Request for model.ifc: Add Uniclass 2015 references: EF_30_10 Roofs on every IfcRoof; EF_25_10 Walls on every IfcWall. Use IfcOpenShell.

First a look at what the model holds.

```python
import ifcopenshell

model = ifcopenshell.open("model.ifc")
print(model.schema)
print("classifications:", [c.Name for c in model.by_type("IfcClassification")])
for ifc_class in ("IfcDoor", "IfcRoof", "IfcStair", "IfcWall", "IfcWindow"):
    print(ifc_class, len(model.by_type(ifc_class)))
```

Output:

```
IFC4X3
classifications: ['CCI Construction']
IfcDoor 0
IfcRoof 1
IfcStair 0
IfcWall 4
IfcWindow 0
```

```python
import ifcopenshell
import ifcopenshell.api.classification

model = ifcopenshell.open("model.ifc")

system = ifcopenshell.api.classification.add_classification(model, classification="Uniclass 2015")

codes = {
    "IfcRoof": ("EF_30_10", "Roofs"),
    "IfcWall": ("EF_25_10", "Walls"),
}
for ifc_class, (code, name) in codes.items():
    products = model.by_type(ifc_class)
    ifcopenshell.api.classification.add_reference(
        model, products=products, classification=system, identification=code, name=name
    )
    print(code, len(products))

model.write("model_edited.ifc")
```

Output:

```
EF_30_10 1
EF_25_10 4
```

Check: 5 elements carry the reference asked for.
